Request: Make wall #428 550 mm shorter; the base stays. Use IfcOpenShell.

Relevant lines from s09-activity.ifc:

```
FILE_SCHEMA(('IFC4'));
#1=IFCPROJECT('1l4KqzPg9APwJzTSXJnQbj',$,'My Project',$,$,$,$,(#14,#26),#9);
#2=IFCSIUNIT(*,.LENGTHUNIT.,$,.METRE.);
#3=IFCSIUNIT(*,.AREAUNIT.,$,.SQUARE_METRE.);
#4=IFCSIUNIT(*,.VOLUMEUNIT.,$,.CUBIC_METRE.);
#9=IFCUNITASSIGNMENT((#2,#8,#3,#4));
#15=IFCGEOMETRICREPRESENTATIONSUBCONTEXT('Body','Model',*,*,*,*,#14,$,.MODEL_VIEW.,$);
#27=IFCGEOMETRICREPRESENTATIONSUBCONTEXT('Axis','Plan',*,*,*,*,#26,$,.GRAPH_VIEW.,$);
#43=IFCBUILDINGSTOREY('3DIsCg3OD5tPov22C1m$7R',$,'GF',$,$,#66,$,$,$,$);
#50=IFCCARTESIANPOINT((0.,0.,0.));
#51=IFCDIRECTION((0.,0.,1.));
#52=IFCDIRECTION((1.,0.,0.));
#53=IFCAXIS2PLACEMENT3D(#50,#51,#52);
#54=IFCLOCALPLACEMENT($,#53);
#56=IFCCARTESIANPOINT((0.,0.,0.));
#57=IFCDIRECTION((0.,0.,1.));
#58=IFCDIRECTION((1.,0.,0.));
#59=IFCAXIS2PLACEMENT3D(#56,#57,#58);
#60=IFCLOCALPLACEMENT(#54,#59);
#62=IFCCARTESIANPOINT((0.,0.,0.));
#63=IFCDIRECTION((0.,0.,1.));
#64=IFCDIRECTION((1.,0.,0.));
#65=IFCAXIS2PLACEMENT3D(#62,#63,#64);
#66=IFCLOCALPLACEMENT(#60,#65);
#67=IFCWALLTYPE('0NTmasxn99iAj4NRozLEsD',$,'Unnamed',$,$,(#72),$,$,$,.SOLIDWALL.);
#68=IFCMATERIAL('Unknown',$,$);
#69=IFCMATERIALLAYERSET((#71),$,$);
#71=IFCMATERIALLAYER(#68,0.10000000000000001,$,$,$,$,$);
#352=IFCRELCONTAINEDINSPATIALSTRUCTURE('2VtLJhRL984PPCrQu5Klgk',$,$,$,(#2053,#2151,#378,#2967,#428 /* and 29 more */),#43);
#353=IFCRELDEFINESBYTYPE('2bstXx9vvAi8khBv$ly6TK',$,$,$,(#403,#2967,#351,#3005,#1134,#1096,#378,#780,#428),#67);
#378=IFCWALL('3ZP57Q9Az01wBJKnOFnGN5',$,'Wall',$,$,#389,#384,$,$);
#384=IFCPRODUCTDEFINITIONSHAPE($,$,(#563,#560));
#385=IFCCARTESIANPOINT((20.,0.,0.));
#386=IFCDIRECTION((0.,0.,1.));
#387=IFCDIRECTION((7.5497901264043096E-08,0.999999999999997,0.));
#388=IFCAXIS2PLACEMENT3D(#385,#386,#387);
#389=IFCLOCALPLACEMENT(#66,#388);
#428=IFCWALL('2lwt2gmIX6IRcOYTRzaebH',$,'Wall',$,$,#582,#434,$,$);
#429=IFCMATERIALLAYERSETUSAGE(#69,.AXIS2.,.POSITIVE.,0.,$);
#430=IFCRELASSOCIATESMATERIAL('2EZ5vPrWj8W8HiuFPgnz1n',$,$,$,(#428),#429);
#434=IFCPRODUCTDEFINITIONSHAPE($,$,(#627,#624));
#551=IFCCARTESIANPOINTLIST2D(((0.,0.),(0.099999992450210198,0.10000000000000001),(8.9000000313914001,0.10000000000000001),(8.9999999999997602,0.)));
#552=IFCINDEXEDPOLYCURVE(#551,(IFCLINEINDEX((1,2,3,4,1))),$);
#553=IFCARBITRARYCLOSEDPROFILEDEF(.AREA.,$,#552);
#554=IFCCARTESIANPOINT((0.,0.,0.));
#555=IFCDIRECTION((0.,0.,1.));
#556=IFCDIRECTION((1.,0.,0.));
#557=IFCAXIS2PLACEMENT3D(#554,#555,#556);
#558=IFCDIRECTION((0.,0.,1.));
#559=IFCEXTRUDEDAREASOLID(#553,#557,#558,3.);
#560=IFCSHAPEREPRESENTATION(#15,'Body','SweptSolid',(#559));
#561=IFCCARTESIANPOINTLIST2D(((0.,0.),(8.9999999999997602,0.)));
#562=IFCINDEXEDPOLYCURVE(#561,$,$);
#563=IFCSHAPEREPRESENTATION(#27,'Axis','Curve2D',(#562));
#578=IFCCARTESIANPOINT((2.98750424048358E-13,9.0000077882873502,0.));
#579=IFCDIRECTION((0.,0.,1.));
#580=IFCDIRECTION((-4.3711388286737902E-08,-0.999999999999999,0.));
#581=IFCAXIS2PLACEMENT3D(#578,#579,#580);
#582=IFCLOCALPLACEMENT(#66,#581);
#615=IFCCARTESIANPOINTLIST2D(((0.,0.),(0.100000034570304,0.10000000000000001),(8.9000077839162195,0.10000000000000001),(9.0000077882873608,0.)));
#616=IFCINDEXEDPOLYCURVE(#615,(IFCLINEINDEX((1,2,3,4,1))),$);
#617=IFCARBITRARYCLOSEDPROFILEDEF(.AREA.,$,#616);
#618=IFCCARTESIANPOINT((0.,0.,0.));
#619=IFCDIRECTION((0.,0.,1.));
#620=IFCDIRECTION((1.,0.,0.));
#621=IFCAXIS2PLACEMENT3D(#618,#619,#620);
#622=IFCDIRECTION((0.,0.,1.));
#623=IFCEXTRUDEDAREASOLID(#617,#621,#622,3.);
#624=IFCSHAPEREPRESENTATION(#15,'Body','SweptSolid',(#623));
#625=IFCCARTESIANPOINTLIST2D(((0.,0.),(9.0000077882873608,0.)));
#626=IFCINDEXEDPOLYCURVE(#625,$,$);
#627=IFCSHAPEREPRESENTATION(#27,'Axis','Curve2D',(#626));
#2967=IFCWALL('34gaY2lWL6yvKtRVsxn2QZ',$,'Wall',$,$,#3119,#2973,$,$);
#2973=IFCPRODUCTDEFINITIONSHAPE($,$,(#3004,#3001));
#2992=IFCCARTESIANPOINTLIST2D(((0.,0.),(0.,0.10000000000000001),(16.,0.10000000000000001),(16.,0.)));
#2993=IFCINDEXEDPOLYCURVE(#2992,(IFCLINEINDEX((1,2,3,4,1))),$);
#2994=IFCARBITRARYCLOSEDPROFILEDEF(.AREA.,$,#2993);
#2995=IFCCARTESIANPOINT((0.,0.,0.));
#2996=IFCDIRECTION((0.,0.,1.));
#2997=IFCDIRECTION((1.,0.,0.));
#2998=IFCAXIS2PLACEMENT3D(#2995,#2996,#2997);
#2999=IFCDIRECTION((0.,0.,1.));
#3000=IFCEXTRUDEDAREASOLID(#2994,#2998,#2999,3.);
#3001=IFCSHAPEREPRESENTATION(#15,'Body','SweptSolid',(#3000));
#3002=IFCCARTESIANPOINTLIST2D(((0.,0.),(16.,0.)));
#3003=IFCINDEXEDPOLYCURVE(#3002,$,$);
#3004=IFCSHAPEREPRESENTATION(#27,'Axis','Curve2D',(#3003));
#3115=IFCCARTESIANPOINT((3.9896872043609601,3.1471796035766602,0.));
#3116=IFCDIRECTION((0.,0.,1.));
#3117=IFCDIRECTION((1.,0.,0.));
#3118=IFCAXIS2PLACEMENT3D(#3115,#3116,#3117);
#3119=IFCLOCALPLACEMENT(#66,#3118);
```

```python
import ifcopenshell
import ifcopenshell.geom
import ifcopenshell.util.representation
import ifcopenshell.util.shape

model = ifcopenshell.open("s09-activity.ifc")
settings = ifcopenshell.geom.settings()


def volume(element):
    """Net volume in cubic metres, openings subtracted."""
    shape = ifcopenshell.geom.create_shape(settings, element)
    return ifcopenshell.util.shape.get_volume(shape.geometry)


wall = model.by_guid("2lwt2gmIX6IRcOYTRzaebH")
before = volume(wall)

body = ifcopenshell.util.representation.get_representation(wall, "Model", "Body")
solid = body.Items[0]
old_height = solid.Depth
solid.Depth -= 0.55
after = volume(wall)

print(f"height {old_height:g} -> {solid.Depth:g}, volume {before:.3f} -> {after:.3f} m3")

model.write("s09-activity_edited.ifc")
```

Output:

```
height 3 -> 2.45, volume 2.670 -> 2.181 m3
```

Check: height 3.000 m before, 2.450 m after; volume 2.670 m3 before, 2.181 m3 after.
